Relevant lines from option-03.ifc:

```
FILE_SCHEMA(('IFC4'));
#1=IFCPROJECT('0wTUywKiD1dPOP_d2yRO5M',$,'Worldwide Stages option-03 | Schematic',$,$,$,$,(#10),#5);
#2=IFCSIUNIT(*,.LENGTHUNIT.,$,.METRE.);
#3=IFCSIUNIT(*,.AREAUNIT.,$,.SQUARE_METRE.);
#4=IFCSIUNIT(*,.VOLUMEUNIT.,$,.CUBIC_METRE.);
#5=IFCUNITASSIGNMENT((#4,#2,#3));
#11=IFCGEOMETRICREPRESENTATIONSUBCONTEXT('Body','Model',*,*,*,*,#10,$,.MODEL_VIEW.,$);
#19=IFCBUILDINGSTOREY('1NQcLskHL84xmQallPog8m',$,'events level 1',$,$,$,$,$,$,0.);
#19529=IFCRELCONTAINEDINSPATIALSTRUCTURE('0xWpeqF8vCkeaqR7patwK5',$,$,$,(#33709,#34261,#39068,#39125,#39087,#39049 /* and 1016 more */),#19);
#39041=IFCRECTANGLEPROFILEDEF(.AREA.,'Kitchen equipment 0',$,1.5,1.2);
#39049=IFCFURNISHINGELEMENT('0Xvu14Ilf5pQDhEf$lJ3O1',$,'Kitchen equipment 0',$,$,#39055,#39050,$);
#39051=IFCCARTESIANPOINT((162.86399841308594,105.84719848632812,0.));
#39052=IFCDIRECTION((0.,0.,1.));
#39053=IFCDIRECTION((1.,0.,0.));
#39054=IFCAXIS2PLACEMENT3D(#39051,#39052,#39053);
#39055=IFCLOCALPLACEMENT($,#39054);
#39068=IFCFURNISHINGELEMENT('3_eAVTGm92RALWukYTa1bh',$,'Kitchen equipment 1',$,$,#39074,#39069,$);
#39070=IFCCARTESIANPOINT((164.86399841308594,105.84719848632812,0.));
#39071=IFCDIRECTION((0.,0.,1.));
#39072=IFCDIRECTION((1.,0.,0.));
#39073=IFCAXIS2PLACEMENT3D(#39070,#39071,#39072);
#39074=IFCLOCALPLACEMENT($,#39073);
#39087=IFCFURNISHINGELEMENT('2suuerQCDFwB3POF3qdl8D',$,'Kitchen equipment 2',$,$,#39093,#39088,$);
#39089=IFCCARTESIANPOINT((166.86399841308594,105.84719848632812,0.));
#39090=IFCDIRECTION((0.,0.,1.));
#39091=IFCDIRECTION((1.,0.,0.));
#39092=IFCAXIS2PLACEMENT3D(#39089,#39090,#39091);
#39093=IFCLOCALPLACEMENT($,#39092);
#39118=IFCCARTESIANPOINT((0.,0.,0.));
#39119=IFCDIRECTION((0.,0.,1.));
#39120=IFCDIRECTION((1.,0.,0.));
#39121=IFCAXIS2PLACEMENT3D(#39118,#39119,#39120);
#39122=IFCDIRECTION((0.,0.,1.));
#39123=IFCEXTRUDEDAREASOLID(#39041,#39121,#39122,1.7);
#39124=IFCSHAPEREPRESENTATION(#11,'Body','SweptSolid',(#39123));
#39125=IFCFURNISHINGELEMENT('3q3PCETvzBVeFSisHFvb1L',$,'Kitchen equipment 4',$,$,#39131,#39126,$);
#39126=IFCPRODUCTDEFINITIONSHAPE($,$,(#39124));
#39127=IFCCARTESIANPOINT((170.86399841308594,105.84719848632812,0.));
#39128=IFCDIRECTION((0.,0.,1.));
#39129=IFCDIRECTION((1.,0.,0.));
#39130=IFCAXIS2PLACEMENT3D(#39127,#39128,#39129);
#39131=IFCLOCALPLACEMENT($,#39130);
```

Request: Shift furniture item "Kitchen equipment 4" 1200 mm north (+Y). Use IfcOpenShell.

```python
import ifcopenshell
import ifcopenshell.api.geometry
import ifcopenshell.util.placement

model = ifcopenshell.open("option-03.ifc")

item = model.by_guid("3q3PCETvzBVeFSisHFvb1L")
matrix = ifcopenshell.util.placement.get_local_placement(item.ObjectPlacement)
matrix[1, 3] += 1.2
ifcopenshell.api.geometry.edit_object_placement(model, product=item, matrix=matrix, is_si=False)

print(ifcopenshell.util.placement.get_local_placement(item.ObjectPlacement).round(3) + 0.0)

model.write("option-03_v2.ifc")
```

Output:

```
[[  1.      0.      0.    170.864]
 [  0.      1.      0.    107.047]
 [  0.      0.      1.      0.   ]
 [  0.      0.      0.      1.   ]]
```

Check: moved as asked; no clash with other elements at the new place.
